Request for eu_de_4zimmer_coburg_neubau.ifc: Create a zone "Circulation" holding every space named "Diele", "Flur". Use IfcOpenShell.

First a look at what the model holds.

```python
import ifcopenshell

model = ifcopenshell.open("eu_de_4zimmer_coburg_neubau.ifc")
print(model.schema)
seen = {}
for space in model.by_type("IfcSpace"):
    seen[space.LongName] = seen.get(space.LongName, 0) + 1
for name, count in sorted(seen.items(), key=str):
    print(count, "x", name)
print("zones:", [z.Name for z in model.by_type("IfcZone")][:20])
```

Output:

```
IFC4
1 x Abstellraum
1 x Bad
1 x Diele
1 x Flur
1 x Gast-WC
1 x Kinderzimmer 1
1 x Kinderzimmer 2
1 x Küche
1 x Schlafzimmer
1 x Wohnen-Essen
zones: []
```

```python
import ifcopenshell
import ifcopenshell.api.group
import ifcopenshell.api.root

model = ifcopenshell.open("eu_de_4zimmer_coburg_neubau.ifc")

names = {"Diele", "Flur"}
spaces = [s for s in model.by_type("IfcSpace") if s.LongName in names]

zone = ifcopenshell.api.root.create_entity(model, ifc_class="IfcZone", name="Circulation")
ifcopenshell.api.group.assign_group(model, products=spaces, group=zone)
print(len(spaces), "spaces in", zone.Name)

model.write("eu_de_4zimmer_coburg_neubau_v2.ifc")
```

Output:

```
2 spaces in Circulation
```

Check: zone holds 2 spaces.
